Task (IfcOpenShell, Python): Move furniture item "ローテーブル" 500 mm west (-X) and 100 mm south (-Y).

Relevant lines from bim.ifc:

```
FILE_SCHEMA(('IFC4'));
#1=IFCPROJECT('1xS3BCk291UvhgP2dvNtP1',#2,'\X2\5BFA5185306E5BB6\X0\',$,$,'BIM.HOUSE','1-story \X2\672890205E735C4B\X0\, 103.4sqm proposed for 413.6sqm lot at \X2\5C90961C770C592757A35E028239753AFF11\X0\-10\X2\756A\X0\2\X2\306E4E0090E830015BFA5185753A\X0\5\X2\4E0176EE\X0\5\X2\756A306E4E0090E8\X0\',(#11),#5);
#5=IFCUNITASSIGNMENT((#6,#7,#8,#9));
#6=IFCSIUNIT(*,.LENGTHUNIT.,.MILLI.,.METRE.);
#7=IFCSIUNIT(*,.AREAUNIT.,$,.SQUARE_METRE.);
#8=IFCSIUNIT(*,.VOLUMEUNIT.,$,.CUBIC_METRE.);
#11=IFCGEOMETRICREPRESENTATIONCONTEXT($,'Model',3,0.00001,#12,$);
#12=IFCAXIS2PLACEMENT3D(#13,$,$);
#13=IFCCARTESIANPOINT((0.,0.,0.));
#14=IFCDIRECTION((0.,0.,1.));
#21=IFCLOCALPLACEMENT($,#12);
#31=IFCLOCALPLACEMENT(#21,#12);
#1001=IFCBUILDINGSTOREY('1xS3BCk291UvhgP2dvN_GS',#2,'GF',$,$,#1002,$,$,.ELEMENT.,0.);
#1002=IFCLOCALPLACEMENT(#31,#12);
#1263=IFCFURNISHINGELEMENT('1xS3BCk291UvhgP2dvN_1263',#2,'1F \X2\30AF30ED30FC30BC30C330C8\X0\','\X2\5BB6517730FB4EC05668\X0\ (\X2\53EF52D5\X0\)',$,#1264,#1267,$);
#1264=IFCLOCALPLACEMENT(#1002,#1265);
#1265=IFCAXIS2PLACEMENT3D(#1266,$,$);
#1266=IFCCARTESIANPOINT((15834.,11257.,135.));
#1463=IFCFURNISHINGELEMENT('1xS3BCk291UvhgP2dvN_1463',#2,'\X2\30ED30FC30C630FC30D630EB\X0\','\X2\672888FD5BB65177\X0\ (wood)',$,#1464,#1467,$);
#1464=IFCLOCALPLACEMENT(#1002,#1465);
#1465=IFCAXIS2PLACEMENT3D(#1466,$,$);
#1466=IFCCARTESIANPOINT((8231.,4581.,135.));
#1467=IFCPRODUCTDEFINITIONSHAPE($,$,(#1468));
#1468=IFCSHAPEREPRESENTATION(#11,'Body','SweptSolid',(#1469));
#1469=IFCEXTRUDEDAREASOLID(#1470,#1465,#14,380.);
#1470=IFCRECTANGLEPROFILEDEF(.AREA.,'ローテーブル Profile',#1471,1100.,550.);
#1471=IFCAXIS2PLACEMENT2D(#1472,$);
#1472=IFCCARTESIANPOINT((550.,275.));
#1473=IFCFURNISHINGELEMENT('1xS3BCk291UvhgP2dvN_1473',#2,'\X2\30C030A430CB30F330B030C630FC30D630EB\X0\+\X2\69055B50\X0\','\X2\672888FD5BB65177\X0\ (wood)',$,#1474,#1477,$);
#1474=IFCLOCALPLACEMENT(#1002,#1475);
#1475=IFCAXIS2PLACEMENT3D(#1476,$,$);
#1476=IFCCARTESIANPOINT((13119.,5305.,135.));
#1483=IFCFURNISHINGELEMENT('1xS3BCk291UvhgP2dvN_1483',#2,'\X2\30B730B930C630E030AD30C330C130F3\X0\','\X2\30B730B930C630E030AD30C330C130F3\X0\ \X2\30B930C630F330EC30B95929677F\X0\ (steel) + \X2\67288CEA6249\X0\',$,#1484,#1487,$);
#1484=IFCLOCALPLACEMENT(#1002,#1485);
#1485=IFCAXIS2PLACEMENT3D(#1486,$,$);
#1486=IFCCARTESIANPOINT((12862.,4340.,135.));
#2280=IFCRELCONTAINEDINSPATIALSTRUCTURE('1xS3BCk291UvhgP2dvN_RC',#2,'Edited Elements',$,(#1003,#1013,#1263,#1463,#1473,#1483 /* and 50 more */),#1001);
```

```python
import ifcopenshell
import ifcopenshell.api.geometry
import ifcopenshell.util.placement
import ifcopenshell.util.unit

model = ifcopenshell.open("bim.ifc")
unit_scale = ifcopenshell.util.unit.calculate_unit_scale(model)

item = model.by_guid("1xS3BCk291UvhgP2dvN_1463")
matrix = ifcopenshell.util.placement.get_local_placement(item.ObjectPlacement)
matrix[0, 3] -= 0.5 / unit_scale
matrix[1, 3] -= 0.1 / unit_scale
ifcopenshell.api.geometry.edit_object_placement(model, product=item, matrix=matrix, is_si=False)

print(ifcopenshell.util.placement.get_local_placement(item.ObjectPlacement).round(3) + 0.0)

model.write("bim_updated.ifc")
```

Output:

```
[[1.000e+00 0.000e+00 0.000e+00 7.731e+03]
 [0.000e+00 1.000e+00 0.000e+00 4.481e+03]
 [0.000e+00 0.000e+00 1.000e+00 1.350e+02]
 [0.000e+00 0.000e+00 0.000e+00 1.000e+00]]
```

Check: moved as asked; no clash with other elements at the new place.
